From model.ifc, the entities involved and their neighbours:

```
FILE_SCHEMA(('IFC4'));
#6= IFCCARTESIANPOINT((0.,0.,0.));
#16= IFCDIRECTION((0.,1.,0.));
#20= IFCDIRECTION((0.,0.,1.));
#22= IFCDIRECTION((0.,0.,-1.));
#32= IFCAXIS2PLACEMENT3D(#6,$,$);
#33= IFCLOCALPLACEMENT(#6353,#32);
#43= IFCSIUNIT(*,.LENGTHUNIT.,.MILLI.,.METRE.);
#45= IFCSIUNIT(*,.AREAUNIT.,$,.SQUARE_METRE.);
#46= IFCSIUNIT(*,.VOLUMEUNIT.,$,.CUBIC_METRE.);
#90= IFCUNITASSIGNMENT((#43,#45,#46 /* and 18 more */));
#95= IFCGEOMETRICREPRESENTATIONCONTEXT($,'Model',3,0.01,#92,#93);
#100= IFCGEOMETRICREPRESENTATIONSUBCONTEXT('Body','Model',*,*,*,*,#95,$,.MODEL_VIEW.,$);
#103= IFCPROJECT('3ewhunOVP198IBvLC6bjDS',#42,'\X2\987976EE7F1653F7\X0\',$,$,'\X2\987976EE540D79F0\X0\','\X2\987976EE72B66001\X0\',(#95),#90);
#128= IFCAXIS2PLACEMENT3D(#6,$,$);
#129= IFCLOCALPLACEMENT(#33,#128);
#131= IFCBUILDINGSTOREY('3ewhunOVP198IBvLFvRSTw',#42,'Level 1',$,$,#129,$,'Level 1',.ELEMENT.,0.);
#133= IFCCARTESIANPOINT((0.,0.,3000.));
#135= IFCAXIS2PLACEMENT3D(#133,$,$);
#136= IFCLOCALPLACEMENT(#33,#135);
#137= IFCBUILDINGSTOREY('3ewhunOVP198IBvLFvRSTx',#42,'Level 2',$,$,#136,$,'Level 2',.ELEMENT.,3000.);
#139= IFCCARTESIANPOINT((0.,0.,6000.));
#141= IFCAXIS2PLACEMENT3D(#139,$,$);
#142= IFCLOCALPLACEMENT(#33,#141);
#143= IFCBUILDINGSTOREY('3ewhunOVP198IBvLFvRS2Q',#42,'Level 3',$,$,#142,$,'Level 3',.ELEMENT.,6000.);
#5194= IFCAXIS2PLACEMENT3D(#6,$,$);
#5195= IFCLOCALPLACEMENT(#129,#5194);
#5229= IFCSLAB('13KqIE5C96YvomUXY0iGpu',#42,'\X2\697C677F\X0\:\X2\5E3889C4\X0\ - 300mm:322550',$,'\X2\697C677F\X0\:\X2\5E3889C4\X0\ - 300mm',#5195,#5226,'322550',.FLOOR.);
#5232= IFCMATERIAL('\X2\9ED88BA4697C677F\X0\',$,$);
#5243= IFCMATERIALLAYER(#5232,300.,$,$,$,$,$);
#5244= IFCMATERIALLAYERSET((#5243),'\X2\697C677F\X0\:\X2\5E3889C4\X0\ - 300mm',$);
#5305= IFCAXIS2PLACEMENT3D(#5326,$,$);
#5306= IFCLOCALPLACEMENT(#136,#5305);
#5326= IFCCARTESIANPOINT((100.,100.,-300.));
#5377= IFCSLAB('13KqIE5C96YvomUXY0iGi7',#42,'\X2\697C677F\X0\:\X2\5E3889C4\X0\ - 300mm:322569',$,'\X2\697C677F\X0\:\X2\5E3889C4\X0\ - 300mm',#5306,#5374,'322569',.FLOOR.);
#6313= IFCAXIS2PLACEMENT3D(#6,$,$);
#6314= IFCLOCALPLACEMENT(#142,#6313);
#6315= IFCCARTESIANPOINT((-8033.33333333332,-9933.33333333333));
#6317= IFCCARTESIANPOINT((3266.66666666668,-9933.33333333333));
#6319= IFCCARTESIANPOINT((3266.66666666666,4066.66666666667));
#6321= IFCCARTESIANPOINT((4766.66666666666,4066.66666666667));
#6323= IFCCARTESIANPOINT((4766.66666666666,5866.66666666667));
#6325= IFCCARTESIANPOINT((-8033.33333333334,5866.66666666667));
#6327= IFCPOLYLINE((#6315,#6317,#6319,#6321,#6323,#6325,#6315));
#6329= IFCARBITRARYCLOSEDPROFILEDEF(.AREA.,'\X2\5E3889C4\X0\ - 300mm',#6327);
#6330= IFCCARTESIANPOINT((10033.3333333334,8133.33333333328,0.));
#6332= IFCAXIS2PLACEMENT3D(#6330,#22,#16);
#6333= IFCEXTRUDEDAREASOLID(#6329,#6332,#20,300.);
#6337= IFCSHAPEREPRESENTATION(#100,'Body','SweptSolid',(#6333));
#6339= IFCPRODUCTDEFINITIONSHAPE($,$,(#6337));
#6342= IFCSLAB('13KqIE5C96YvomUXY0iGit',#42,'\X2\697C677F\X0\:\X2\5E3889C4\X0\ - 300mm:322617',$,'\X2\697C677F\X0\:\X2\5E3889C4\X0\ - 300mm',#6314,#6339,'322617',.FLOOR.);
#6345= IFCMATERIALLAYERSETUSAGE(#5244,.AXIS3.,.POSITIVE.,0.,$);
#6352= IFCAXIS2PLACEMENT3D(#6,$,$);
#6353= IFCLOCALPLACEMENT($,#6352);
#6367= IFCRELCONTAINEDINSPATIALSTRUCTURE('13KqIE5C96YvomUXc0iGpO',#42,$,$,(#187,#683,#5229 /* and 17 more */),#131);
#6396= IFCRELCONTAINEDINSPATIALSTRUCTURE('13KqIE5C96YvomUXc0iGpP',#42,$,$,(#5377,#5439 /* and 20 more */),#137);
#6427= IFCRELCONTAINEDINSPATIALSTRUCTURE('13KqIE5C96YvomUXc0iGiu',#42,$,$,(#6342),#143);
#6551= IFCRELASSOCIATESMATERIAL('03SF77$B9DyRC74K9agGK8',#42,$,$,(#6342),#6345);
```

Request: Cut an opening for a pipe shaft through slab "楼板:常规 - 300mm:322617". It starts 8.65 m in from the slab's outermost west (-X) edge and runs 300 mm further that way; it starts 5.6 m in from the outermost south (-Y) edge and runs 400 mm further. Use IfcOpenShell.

```python
import numpy as np
import ifcopenshell
import ifcopenshell.api.feature
import ifcopenshell.api.geometry
import ifcopenshell.api.root
import ifcopenshell.geom
import ifcopenshell.util.placement
import ifcopenshell.util.representation
import ifcopenshell.util.shape
import ifcopenshell.util.unit

model = ifcopenshell.open("model.ifc")
unit_scale = ifcopenshell.util.unit.calculate_unit_scale(model)
settings = ifcopenshell.geom.settings()


def volume(element):
    """Net volume in cubic metres, openings subtracted."""
    shape = ifcopenshell.geom.create_shape(settings, element)
    return ifcopenshell.util.shape.get_volume(shape.geometry)


slab = model.by_guid("13KqIE5C96YvomUXY0iGit")
before = volume(slab)

# Extent in the slab's own axes, in metres. The edges named are its -X and -Y sides.
slab_shape = ifcopenshell.geom.create_shape(settings, slab)
vertices = ifcopenshell.util.shape.get_vertices(slab_shape.geometry)
x_min, y_min, bottom = vertices.min(axis=0)
top = vertices[:, 2].max()

opening = ifcopenshell.api.root.create_entity(model, ifc_class="IfcOpeningElement", name="Pipe shaft opening", predefined_type="OPENING")
context = ifcopenshell.util.representation.get_context(model, "Model", "Body", "MODEL_VIEW")
width, depth = 0.3, 0.4
outline = [(0.0, 0.0), (width, 0.0), (width, depth), (0.0, depth), (0.0, 0.0)]
# Overshoot both faces by 50 mm so the cut is clean.
shape = ifcopenshell.api.geometry.add_slab_representation(
    model, context=context, depth=top - bottom + 0.1, polyline=outline
)
ifcopenshell.api.geometry.assign_representation(model, product=opening, representation=shape)

matrix = ifcopenshell.util.placement.get_local_placement(slab.ObjectPlacement)
matrix[:, 3] = matrix @ np.append(np.array([x_min + 8.65, y_min + 5.6, bottom - 0.05]) / unit_scale, 1.0)
ifcopenshell.api.geometry.edit_object_placement(model, product=opening, matrix=matrix, is_si=False)
ifcopenshell.api.feature.add_feature(model, feature=opening, element=slab)

after = volume(slab)

print(f"slab volume {before:.3f} -> {after:.3f} m3")

model.write("model_updated.ifc")
```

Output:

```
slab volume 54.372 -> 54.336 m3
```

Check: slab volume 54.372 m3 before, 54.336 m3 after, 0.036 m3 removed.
